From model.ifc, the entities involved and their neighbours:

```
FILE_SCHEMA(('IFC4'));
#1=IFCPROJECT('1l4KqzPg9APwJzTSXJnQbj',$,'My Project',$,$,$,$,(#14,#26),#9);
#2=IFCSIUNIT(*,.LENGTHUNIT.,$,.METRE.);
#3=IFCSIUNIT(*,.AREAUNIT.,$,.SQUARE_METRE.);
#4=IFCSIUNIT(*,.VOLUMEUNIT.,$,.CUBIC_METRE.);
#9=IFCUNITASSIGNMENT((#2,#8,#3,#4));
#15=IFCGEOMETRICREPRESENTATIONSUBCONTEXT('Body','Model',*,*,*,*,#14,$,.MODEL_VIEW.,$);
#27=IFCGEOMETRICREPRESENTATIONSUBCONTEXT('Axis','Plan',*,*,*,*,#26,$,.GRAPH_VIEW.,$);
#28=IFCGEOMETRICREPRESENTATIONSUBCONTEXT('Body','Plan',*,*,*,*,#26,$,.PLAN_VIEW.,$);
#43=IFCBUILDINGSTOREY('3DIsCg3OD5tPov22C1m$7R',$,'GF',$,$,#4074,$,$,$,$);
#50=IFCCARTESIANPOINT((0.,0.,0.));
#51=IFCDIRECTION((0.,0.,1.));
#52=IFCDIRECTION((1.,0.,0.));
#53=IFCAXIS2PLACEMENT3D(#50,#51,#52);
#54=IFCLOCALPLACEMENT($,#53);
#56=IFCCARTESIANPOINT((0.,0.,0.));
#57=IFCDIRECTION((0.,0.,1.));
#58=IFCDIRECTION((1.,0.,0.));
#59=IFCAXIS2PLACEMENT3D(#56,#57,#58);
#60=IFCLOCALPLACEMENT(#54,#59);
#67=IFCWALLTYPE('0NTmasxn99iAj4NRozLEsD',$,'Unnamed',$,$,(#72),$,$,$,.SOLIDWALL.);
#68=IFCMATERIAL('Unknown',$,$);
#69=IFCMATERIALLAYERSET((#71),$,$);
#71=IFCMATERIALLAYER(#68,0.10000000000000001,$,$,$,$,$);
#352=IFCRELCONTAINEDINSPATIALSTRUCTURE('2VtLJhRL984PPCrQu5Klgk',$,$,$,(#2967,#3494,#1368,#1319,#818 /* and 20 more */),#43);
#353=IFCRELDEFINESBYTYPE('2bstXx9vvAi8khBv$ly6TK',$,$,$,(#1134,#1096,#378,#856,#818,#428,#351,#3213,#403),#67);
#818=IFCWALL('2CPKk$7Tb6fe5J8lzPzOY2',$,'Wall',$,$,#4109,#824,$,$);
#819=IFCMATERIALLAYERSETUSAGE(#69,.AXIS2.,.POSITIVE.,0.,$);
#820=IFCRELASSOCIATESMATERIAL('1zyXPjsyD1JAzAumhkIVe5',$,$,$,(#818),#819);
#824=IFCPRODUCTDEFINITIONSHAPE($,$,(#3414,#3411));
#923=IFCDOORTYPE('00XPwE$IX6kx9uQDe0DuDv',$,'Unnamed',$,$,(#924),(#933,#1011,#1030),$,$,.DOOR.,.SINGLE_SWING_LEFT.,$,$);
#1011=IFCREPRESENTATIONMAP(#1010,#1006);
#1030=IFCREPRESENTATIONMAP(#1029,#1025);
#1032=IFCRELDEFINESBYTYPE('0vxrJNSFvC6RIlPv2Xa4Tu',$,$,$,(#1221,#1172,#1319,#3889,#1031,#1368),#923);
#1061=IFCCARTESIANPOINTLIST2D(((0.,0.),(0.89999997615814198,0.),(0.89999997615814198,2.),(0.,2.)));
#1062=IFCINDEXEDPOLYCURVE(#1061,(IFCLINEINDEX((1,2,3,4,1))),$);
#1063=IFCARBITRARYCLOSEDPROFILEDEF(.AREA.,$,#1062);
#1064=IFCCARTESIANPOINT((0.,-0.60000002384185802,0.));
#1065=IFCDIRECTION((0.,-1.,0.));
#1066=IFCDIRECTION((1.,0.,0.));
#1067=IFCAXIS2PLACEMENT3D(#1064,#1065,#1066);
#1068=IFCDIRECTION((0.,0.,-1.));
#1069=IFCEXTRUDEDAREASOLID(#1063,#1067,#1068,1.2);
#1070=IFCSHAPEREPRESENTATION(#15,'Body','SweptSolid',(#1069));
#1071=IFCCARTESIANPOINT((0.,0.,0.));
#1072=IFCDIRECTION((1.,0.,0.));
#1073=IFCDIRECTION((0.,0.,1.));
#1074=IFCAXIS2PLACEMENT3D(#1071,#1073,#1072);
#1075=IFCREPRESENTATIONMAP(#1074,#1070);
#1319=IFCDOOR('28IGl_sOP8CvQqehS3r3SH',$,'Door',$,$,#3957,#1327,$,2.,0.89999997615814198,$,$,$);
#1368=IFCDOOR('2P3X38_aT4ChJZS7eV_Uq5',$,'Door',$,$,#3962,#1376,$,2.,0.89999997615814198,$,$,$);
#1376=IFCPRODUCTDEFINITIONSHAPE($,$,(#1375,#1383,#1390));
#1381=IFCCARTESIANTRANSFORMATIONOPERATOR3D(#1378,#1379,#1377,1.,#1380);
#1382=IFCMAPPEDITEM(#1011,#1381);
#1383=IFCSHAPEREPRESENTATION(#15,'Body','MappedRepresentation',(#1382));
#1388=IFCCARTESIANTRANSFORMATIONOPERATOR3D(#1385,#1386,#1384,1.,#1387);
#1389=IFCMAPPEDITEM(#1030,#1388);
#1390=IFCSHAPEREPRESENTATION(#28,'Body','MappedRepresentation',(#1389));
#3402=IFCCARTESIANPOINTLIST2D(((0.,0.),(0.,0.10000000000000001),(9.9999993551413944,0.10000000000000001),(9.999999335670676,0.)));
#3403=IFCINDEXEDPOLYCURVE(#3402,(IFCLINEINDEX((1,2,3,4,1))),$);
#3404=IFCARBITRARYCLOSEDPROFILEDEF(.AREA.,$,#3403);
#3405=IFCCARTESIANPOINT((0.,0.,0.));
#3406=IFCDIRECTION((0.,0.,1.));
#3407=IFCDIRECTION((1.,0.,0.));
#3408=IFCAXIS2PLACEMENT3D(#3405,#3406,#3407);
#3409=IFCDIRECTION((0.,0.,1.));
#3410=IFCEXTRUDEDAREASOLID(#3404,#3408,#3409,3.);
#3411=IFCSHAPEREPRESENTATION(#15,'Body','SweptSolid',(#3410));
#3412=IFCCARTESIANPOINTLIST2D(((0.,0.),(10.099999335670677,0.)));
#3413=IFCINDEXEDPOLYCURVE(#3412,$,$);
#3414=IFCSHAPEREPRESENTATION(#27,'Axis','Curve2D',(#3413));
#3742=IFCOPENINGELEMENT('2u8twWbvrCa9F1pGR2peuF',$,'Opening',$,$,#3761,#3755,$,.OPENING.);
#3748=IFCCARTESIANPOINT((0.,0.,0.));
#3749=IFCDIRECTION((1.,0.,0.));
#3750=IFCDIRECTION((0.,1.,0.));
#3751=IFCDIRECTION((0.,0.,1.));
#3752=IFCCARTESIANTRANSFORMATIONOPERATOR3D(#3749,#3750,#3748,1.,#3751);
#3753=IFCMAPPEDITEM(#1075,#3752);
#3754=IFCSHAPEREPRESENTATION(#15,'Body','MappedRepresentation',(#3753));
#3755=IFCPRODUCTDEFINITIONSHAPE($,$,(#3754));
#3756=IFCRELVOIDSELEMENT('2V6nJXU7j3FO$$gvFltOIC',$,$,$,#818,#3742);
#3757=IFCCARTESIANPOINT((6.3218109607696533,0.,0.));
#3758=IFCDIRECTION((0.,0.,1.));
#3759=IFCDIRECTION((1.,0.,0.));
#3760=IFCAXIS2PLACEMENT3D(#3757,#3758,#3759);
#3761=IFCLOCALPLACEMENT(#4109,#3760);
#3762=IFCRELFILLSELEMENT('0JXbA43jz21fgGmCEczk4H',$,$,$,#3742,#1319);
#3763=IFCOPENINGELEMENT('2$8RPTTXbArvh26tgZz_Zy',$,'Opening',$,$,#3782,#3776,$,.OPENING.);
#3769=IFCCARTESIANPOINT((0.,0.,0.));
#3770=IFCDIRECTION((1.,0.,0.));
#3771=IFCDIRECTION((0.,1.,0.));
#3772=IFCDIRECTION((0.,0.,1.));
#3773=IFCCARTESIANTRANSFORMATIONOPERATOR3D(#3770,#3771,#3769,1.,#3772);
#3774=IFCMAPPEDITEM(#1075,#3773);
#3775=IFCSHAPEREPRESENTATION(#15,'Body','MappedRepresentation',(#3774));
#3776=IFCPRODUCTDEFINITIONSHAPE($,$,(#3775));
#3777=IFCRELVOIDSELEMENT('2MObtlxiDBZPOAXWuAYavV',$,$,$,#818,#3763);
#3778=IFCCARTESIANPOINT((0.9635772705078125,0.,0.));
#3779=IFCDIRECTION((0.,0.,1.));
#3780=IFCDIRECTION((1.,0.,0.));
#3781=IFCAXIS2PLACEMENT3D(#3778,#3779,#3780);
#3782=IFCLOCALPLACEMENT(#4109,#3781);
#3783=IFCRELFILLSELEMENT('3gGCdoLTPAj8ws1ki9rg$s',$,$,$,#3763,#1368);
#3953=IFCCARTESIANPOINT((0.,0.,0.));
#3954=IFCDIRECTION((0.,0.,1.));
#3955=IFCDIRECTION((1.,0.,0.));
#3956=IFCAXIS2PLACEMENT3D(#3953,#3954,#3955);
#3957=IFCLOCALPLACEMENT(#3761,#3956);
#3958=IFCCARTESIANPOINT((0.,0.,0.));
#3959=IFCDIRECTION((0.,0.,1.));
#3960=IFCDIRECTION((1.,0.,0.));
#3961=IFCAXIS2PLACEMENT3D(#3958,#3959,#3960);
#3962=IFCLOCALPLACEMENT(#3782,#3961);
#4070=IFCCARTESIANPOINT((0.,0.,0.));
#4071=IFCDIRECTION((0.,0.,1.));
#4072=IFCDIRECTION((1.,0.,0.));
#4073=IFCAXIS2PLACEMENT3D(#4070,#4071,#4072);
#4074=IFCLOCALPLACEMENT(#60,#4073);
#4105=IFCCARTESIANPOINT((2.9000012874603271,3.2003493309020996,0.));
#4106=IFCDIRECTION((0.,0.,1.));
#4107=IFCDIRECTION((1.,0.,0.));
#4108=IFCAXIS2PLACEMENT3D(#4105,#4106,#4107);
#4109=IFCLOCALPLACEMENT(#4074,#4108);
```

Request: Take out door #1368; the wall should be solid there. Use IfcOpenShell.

```python
import ifcopenshell
import ifcopenshell.api.feature
import ifcopenshell.api.root
import ifcopenshell.geom
import ifcopenshell.util.shape

model = ifcopenshell.open("model.ifc")
settings = ifcopenshell.geom.settings()


def volume(element):
    """Net volume in cubic metres, openings subtracted."""
    shape = ifcopenshell.geom.create_shape(settings, element)
    return ifcopenshell.util.shape.get_volume(shape.geometry)


door = model.by_guid("2P3X38_aT4ChJZS7eV_Uq5")
opening = door.FillsVoids[0].RelatingOpeningElement
wall = opening.VoidsElements[0].RelatingBuildingElement
before = volume(wall)

ifcopenshell.api.root.remove_product(model, product=door)
ifcopenshell.api.feature.remove_feature(model, feature=opening)

after = volume(wall)

print(f"wall volume {before:.3f} -> {after:.3f} m3")

model.write("model_updated.ifc")
```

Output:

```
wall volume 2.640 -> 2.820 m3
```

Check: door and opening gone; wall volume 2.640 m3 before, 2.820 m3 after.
